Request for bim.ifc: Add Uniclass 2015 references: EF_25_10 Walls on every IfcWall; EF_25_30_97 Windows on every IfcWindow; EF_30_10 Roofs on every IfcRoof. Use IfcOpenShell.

First a look at what the model holds.

```python
import ifcopenshell

model = ifcopenshell.open("bim.ifc")
print(model.schema)
print("classifications:", [c.Name for c in model.by_type("IfcClassification")])
for ifc_class in ("IfcDoor", "IfcRoof", "IfcStair", "IfcWall", "IfcWindow"):
    print(ifc_class, len(model.by_type(ifc_class)))
```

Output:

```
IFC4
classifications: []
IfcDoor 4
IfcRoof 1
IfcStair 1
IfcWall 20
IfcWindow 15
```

```python
import ifcopenshell
import ifcopenshell.api.classification

model = ifcopenshell.open("bim.ifc")

system = ifcopenshell.api.classification.add_classification(model, classification="Uniclass 2015")

codes = {
    "IfcWall": ("EF_25_10", "Walls"),
    "IfcWindow": ("EF_25_30_97", "Windows"),
    "IfcRoof": ("EF_30_10", "Roofs"),
}
for ifc_class, (code, name) in codes.items():
    products = model.by_type(ifc_class)
    ifcopenshell.api.classification.add_reference(
        model, products=products, classification=system, identification=code, name=name
    )
    print(code, len(products))

model.write("bim_v2.ifc")
```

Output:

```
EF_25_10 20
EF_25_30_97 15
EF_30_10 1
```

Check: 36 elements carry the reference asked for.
